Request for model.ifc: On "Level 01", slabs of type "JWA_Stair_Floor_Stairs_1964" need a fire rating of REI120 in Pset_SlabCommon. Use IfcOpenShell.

First a look at what the model holds.

```python
import ifcopenshell
import ifcopenshell.util.element

model = ifcopenshell.open("model.ifc")
print(model.schema)
storey = next(s for s in model.by_type("IfcBuildingStorey") if s.Name == "Level 01")
slabs = [e for e in ifcopenshell.util.element.get_decomposition(storey) if e.is_a("IfcSlab")]
seen = {}
for e in slabs:
    element_type = ifcopenshell.util.element.get_type(e)
    key = (element_type.Name if element_type != e and element_type else None, ifcopenshell.util.element.get_pset(e, "Pset_SlabCommon", "FireRating"))
    seen[key] = seen.get(key, 0) + 1
for (name, value), count in sorted(seen.items(), key=str):
    print(count, "x", name, "|", value)
```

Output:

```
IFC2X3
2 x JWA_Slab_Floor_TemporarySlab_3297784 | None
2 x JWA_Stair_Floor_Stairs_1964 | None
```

```python
import ifcopenshell
import ifcopenshell.api.pset
import ifcopenshell.util.element

model = ifcopenshell.open("model.ifc")

storey = next(s for s in model.by_type("IfcBuildingStorey") if s.Name == "Level 01")
slabs = [e for e in ifcopenshell.util.element.get_decomposition(storey) if e.is_a("IfcSlab")]

count = 0
for e in slabs:
    element_type = ifcopenshell.util.element.get_type(e)
    if element_type in (None, e) or element_type.Name != "JWA_Stair_Floor_Stairs_1964":
        continue
    # add_pset returns the element's existing set when there is one.
    pset = ifcopenshell.api.pset.add_pset(model, product=e, name="Pset_SlabCommon")
    ifcopenshell.api.pset.edit_pset(model, pset=pset, properties={"FireRating": "REI120"})
    count += 1

print(count, "slabs updated")

model.write("model-out.ifc")
```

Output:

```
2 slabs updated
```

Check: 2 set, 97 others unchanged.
